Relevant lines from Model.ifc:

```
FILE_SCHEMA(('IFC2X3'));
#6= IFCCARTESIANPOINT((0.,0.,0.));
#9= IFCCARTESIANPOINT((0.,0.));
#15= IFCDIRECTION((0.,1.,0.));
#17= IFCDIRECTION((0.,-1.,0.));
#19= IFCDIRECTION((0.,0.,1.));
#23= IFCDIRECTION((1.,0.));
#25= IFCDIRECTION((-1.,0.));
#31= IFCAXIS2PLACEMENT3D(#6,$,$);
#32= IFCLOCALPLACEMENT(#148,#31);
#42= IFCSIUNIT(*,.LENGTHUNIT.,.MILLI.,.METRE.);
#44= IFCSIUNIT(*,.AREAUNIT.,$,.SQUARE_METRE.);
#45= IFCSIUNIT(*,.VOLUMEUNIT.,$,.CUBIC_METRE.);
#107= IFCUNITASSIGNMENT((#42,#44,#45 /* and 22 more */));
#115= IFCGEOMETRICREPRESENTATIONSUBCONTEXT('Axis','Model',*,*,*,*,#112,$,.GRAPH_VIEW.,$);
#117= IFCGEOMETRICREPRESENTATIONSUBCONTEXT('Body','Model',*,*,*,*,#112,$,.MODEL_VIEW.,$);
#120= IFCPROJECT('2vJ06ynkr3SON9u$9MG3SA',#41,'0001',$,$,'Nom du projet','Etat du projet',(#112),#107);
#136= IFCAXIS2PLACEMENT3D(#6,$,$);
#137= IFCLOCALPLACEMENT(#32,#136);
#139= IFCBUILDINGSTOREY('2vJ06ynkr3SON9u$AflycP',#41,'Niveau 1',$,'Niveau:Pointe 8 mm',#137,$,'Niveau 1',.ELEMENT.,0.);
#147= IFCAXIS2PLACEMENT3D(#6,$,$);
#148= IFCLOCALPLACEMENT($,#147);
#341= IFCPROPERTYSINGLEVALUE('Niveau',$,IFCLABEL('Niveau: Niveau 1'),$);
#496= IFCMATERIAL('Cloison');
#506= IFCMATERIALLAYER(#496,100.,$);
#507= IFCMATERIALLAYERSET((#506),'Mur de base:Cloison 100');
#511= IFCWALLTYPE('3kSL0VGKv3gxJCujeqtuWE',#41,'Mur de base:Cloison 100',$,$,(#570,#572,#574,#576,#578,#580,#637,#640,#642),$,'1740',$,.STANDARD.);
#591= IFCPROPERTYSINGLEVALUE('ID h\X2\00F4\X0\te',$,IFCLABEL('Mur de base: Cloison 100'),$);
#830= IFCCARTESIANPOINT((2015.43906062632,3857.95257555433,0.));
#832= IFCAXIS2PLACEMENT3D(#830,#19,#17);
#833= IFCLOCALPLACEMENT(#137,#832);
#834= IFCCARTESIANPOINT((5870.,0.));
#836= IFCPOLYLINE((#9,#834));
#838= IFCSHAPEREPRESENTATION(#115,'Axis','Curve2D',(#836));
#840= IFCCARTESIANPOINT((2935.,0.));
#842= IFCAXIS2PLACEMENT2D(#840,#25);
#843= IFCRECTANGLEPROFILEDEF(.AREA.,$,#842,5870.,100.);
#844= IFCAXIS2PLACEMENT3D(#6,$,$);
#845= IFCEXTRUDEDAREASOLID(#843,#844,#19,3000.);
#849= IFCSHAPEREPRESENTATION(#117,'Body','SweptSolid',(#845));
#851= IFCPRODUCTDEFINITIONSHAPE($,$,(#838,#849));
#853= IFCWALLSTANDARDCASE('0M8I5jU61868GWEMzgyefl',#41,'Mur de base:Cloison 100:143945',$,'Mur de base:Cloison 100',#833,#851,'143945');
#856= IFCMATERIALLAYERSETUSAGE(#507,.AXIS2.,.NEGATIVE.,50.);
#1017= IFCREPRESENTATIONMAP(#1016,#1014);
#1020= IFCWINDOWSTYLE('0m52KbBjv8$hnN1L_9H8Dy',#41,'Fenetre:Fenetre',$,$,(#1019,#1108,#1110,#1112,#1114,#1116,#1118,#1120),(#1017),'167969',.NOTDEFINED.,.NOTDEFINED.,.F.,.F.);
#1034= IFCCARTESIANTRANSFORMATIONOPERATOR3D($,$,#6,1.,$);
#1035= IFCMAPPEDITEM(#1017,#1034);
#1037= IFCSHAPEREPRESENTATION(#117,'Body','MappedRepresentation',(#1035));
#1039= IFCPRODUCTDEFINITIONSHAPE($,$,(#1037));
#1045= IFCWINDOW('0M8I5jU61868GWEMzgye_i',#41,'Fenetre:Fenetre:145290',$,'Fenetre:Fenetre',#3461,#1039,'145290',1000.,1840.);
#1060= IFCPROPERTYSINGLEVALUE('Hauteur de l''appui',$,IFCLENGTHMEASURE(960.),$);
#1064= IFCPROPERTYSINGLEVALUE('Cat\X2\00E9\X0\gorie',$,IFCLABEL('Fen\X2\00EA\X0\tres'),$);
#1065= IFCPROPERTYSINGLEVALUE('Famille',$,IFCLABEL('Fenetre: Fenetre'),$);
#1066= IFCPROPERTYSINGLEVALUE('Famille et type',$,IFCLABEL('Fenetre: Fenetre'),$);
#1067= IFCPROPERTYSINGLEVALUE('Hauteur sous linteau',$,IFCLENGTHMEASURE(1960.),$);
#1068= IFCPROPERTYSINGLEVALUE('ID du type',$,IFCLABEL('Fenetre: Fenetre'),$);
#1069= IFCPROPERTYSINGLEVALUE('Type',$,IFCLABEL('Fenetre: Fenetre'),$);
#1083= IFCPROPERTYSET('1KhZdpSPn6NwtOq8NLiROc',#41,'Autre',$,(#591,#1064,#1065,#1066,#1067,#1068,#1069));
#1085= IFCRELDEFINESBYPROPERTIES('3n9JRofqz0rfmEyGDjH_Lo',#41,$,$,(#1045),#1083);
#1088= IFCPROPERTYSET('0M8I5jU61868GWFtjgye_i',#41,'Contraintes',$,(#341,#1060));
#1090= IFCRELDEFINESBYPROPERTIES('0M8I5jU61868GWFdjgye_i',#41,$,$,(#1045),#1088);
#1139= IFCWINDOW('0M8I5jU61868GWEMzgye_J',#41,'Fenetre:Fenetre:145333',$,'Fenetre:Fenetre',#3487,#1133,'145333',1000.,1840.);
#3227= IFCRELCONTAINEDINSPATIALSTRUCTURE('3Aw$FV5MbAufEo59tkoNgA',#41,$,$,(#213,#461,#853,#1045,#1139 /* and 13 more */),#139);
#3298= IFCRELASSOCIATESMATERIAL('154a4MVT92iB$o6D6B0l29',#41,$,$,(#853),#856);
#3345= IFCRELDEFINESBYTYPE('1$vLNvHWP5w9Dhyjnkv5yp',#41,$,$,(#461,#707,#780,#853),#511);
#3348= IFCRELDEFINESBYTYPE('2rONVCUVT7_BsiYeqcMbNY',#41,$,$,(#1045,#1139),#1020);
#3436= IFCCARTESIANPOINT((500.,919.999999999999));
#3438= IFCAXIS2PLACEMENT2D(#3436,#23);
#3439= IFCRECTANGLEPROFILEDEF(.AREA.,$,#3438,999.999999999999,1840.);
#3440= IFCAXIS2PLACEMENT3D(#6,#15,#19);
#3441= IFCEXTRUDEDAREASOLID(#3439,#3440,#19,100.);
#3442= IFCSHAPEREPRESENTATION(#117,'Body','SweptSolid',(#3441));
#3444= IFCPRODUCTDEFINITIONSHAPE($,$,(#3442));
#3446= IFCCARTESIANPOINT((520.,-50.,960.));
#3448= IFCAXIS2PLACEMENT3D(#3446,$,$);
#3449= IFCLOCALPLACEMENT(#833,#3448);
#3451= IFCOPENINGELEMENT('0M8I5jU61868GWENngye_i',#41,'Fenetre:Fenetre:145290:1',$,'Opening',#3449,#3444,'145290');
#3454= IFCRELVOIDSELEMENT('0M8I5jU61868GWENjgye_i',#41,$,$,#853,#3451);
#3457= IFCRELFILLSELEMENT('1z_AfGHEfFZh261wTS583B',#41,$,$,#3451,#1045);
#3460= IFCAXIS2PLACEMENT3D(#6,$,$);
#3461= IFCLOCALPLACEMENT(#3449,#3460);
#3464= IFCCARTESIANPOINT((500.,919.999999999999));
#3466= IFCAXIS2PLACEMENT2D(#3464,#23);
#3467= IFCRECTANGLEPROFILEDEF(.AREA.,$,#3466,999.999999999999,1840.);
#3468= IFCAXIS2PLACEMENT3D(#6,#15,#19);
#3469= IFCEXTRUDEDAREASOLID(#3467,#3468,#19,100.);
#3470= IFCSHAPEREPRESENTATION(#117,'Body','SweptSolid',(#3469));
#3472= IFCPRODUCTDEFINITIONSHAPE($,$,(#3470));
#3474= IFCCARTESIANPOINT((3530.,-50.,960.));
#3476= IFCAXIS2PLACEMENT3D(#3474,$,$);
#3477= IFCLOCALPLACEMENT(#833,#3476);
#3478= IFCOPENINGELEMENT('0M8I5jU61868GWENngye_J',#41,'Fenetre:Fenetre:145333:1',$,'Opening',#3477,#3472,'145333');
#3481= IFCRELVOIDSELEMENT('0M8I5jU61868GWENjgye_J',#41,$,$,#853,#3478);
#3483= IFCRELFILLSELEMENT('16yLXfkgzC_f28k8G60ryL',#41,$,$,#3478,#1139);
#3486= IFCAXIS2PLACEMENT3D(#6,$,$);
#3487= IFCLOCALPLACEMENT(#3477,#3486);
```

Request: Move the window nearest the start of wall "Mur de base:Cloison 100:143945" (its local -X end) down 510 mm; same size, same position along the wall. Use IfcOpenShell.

```python
import numpy as np
import ifcopenshell
import ifcopenshell.api.geometry
import ifcopenshell.api.pset
import ifcopenshell.util.element
import ifcopenshell.util.placement
import ifcopenshell.util.unit

model = ifcopenshell.open("Model.ifc")
unit_scale = ifcopenshell.util.unit.calculate_unit_scale(model)

window = model.by_guid("0M8I5jU61868GWEMzgye_i")
opening = window.FillsVoids[0].RelatingOpeningElement
dz = -510.0

shift = np.array([0.0, 0.0, dz])
# The window is placed relative to its opening, so it follows when the opening moves.
matrix = ifcopenshell.util.placement.get_local_placement(opening.ObjectPlacement)
matrix[:3, 3] += shift
ifcopenshell.api.geometry.edit_object_placement(
    model, product=opening, matrix=matrix, is_si=False, should_transform_children=True
)

# Keep the stored heights in step.
pset = model.by_id(ifcopenshell.util.element.get_pset(window, "Autre", should_inherit=False)["id"])
ifcopenshell.api.pset.edit_pset(model, pset=pset, properties={
    "Hauteur sous linteau": model.create_entity("IfcLengthMeasure", ifcopenshell.util.element.get_pset(window, "Autre", "Hauteur sous linteau") + dz),
})
pset = model.by_id(ifcopenshell.util.element.get_pset(window, "Contraintes", should_inherit=False)["id"])
ifcopenshell.api.pset.edit_pset(model, pset=pset, properties={
    "Hauteur de l'appui": model.create_entity("IfcLengthMeasure", ifcopenshell.util.element.get_pset(window, "Contraintes", "Hauteur de l'appui") + dz),
})

print(f"moved by {dz * unit_scale:+.3f} m")

model.write("Model-out.ifc")
```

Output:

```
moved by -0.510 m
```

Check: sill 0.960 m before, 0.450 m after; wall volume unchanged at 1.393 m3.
